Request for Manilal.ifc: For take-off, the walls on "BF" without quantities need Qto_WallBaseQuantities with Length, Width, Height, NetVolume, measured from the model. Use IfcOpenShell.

First a look at what the model holds.

```python
import ifcopenshell
import ifcopenshell.util.element
import ifcopenshell.util.unit

model = ifcopenshell.open("Manilal.ifc")
print(model.schema)
for unit_type in ("LENGTHUNIT", "AREAUNIT", "VOLUMEUNIT"):
    print(unit_type, ifcopenshell.util.unit.calculate_unit_scale(model, unit_type))
storey = next(s for s in model.by_type("IfcBuildingStorey") if s.Name == "BF")
walls = [e for e in ifcopenshell.util.element.get_decomposition(storey) if e.is_a("IfcWall")]
for e in sorted(walls, key=lambda e: e.id()):
    print(e.id(), e.is_a(), e.Name, list(ifcopenshell.util.element.get_psets(e, qtos_only=True)), sep=" | ")
```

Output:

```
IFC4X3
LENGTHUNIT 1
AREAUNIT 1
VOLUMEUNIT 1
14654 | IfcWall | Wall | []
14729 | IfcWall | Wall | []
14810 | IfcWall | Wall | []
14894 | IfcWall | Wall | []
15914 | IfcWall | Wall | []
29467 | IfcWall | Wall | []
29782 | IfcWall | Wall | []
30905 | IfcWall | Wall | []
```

```python
import ifcopenshell
import ifcopenshell.api.pset
import ifcopenshell.geom
import ifcopenshell.util.element
import ifcopenshell.util.shape
import ifcopenshell.util.unit

model = ifcopenshell.open("Manilal.ifc")
unit_scale = ifcopenshell.util.unit.calculate_unit_scale(model)
volume_scale = ifcopenshell.util.unit.calculate_unit_scale(model, "VOLUMEUNIT")
settings = ifcopenshell.geom.settings()

storey = next(s for s in model.by_type("IfcBuildingStorey") if s.Name == "BF")
walls = [e for e in ifcopenshell.util.element.get_decomposition(storey) if e.is_a("IfcWall")]

for e in sorted(walls, key=lambda e: e.id()):
    if ifcopenshell.util.element.get_psets(e, qtos_only=True, should_inherit=False):
        continue
    # Geometry comes back in metres, in the element's own axes.
    shape = ifcopenshell.geom.create_shape(settings, e)
    values = {
        "Length": ifcopenshell.util.shape.get_x(shape.geometry) / unit_scale,
        "Width": ifcopenshell.util.shape.get_y(shape.geometry) / unit_scale,
        "Height": ifcopenshell.util.shape.get_z(shape.geometry) / unit_scale,
        "NetVolume": ifcopenshell.util.shape.get_volume(shape.geometry) / volume_scale,
    }
    qto = ifcopenshell.api.pset.add_qto(model, product=e, name="Qto_WallBaseQuantities")
    ifcopenshell.api.pset.edit_qto(model, qto=qto, properties=values)
    print(e.id(), {k: round(v, 3) for k, v in values.items()})

model.write("Manilal-out.ifc")
```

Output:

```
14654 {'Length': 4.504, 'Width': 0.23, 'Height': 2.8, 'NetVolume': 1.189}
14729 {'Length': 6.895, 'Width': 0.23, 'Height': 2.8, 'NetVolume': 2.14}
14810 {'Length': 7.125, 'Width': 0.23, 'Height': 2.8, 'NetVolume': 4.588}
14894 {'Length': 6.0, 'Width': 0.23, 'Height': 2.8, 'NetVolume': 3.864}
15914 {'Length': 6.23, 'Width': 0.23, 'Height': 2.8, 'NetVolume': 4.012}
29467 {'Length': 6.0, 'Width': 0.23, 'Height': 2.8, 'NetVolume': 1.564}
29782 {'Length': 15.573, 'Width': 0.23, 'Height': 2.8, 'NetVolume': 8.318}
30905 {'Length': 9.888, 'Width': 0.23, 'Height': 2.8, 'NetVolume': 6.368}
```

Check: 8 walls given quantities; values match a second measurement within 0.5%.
